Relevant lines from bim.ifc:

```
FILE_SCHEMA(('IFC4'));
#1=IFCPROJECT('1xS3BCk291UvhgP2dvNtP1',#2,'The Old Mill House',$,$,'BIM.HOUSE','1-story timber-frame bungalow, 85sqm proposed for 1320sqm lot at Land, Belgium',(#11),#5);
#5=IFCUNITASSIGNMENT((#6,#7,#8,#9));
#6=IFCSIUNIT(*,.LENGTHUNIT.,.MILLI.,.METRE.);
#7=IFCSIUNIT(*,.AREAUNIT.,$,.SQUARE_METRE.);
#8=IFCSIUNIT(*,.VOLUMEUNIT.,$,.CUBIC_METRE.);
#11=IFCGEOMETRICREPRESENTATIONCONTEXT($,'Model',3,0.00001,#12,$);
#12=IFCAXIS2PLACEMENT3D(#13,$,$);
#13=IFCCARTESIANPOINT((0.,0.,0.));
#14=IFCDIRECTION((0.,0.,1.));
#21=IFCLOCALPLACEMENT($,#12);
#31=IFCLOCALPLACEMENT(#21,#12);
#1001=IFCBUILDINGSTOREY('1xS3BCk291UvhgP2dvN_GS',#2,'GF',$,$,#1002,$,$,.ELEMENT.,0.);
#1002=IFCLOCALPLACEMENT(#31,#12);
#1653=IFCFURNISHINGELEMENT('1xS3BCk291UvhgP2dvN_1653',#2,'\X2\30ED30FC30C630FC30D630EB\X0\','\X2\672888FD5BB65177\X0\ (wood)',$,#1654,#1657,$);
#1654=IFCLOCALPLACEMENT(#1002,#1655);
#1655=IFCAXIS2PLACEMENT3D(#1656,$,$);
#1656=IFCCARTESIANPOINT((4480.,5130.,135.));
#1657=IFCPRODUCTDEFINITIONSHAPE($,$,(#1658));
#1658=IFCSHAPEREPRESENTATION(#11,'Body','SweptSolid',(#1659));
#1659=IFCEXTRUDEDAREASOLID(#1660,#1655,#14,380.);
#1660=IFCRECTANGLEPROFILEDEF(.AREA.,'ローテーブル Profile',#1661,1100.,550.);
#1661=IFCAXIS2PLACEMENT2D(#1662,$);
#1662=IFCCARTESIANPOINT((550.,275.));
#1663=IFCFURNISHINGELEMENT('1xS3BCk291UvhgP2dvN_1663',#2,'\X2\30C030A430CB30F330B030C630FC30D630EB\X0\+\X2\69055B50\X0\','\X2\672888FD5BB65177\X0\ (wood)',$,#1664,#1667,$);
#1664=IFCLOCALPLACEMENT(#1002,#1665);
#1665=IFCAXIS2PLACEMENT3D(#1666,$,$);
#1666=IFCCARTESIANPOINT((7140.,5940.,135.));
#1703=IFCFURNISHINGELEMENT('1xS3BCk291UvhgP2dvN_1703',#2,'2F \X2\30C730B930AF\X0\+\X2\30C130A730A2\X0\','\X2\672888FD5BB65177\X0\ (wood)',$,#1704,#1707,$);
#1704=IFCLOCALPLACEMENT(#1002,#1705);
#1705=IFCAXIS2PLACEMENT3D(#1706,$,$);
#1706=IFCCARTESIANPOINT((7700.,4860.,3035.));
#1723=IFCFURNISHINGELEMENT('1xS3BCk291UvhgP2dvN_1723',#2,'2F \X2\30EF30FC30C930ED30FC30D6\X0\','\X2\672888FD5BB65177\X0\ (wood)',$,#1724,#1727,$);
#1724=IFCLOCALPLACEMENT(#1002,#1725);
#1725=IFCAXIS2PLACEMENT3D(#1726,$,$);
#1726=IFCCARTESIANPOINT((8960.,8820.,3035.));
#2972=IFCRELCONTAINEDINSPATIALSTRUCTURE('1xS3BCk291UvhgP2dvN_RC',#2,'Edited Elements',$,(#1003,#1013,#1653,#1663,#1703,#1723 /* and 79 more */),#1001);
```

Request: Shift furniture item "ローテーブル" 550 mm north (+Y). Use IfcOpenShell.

```python
import ifcopenshell
import ifcopenshell.api.geometry
import ifcopenshell.util.placement
import ifcopenshell.util.unit

model = ifcopenshell.open("bim.ifc")
unit_scale = ifcopenshell.util.unit.calculate_unit_scale(model)

item = model.by_guid("1xS3BCk291UvhgP2dvN_1653")
matrix = ifcopenshell.util.placement.get_local_placement(item.ObjectPlacement)
matrix[1, 3] += 0.55 / unit_scale
ifcopenshell.api.geometry.edit_object_placement(model, product=item, matrix=matrix, is_si=False)

print(ifcopenshell.util.placement.get_local_placement(item.ObjectPlacement).round(3) + 0.0)

model.write("bim-out.ifc")
```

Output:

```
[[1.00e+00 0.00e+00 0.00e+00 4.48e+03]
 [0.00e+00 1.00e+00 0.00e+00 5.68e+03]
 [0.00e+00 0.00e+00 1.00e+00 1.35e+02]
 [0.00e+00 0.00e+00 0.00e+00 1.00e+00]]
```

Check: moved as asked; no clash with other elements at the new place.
